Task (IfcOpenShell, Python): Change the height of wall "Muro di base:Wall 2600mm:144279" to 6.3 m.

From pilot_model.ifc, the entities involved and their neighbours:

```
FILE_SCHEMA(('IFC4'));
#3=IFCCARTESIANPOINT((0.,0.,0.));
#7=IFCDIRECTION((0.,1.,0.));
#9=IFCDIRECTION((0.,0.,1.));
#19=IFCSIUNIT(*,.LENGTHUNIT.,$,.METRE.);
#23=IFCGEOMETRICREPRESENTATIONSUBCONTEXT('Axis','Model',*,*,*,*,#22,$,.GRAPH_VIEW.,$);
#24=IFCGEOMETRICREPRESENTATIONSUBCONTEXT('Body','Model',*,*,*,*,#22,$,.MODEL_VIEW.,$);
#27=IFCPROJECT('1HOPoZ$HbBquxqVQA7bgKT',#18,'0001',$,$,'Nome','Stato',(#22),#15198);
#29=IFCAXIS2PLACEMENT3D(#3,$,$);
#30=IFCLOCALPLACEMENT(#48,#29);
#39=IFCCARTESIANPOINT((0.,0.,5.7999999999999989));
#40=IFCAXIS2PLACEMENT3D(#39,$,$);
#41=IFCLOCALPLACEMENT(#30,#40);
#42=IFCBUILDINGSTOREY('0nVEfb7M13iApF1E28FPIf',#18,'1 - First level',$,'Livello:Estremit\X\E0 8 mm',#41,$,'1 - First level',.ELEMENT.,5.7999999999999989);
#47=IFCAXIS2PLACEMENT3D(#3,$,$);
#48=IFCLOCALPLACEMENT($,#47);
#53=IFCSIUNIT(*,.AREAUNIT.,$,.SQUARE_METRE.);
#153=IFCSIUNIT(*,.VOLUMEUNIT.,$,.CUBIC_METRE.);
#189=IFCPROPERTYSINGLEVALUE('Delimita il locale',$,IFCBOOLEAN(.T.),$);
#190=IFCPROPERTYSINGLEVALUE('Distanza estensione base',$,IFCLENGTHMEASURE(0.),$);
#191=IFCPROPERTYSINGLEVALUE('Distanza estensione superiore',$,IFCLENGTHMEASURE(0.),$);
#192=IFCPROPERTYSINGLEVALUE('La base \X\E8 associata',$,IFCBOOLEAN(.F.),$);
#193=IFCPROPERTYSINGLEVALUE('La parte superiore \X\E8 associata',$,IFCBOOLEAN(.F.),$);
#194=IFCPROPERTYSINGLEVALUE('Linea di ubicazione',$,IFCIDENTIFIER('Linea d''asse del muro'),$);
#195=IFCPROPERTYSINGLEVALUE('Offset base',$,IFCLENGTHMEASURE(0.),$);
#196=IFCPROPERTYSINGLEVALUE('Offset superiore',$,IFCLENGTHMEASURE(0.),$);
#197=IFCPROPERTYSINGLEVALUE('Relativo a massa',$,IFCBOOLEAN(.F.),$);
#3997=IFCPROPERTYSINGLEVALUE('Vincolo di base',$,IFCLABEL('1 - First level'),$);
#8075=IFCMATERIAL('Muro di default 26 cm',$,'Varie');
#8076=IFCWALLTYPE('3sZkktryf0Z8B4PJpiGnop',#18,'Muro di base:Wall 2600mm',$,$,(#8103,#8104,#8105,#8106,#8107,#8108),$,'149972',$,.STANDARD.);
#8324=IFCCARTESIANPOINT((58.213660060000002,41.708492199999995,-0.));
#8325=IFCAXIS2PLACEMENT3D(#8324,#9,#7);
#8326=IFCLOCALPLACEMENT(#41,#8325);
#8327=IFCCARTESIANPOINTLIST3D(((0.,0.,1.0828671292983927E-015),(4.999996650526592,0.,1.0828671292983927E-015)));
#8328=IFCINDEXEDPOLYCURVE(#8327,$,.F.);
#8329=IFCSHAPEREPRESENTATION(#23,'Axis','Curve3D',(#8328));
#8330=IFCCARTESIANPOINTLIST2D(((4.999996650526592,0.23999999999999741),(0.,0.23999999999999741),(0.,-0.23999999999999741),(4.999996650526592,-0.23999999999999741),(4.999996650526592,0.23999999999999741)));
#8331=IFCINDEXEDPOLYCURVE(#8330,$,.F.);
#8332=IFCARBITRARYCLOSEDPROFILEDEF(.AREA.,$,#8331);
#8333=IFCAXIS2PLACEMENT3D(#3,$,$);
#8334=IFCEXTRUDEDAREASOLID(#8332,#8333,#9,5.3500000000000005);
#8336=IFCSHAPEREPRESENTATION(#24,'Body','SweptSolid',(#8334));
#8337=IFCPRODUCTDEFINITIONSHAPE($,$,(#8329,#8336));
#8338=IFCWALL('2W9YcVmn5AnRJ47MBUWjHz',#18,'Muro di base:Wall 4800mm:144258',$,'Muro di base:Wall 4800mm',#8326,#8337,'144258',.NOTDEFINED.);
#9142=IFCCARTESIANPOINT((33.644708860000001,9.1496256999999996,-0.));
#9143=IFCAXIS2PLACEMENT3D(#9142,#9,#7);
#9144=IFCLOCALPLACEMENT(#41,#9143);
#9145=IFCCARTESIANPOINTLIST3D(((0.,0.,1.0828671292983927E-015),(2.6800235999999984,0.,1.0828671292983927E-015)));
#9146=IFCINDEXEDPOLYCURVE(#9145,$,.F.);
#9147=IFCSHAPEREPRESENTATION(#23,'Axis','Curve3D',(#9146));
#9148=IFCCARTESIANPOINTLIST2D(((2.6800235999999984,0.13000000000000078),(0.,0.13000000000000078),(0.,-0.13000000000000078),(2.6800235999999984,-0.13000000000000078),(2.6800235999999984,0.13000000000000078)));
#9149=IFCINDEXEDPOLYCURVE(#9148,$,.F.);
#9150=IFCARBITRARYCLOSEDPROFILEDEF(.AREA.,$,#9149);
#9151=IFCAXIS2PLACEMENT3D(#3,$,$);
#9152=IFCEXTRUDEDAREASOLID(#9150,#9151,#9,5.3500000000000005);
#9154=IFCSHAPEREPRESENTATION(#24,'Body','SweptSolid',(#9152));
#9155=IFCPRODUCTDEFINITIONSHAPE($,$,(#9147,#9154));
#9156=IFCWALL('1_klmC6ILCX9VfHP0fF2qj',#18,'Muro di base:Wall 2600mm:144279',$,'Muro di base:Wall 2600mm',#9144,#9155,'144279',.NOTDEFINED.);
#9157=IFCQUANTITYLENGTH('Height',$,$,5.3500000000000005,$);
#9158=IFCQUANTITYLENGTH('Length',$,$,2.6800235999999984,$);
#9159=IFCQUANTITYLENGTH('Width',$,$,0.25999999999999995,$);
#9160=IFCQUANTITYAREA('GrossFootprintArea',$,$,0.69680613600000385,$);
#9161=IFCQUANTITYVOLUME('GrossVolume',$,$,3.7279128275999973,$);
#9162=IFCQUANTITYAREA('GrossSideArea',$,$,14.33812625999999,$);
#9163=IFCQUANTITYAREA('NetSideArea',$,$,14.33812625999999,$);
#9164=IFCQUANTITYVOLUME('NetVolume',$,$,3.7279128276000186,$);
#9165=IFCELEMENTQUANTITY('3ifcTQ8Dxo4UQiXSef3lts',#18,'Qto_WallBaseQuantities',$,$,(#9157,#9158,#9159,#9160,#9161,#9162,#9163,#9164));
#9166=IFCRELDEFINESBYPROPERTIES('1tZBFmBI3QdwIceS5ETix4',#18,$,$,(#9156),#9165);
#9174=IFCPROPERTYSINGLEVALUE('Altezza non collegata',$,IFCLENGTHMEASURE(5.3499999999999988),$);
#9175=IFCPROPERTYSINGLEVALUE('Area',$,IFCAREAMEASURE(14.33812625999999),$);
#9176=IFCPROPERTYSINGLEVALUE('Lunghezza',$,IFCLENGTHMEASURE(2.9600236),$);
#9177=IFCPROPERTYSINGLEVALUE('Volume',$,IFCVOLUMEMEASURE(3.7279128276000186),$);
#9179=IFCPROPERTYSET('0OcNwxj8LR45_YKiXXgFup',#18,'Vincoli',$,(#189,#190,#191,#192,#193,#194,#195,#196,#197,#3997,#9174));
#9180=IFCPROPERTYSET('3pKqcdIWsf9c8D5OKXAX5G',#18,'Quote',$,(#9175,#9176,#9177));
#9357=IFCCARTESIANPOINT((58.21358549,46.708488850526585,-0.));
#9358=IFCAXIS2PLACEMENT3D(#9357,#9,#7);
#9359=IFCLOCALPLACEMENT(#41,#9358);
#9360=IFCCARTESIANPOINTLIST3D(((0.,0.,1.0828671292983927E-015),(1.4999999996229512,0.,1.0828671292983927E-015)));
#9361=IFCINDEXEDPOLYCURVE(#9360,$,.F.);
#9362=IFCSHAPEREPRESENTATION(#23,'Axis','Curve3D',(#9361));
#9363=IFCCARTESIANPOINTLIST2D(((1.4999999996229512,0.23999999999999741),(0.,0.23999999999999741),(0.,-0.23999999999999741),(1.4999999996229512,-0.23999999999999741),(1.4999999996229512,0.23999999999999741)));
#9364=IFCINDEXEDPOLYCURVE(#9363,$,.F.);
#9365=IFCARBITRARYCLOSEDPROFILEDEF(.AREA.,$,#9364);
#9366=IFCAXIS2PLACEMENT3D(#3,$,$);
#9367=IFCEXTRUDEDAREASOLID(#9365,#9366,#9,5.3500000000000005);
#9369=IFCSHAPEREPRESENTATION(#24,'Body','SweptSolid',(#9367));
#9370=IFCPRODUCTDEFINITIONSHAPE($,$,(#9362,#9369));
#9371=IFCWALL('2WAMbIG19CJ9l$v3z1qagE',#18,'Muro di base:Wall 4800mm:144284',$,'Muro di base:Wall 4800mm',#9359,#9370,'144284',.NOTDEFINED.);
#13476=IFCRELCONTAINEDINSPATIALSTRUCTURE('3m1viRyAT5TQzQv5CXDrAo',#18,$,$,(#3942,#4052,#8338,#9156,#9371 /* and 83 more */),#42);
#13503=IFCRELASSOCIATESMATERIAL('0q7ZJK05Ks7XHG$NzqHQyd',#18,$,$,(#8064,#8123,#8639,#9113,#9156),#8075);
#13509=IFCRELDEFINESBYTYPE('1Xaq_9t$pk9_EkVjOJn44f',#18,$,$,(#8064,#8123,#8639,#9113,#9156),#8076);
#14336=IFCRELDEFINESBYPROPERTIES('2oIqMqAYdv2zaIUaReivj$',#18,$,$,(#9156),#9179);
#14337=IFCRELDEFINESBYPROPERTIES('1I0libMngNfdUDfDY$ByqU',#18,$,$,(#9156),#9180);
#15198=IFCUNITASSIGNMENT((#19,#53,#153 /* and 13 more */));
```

```python
import ifcopenshell
import ifcopenshell.api.pset
import ifcopenshell.geom
import ifcopenshell.util.element
import ifcopenshell.util.representation
import ifcopenshell.util.shape
import ifcopenshell.util.unit

model = ifcopenshell.open("pilot_model.ifc")
unit_scale = ifcopenshell.util.unit.calculate_unit_scale(model)
area_scale = ifcopenshell.util.unit.calculate_unit_scale(model, "AREAUNIT")
volume_scale = ifcopenshell.util.unit.calculate_unit_scale(model, "VOLUMEUNIT")
settings = ifcopenshell.geom.settings()


def volume(element):
    """Net volume in cubic metres, openings subtracted."""
    shape = ifcopenshell.geom.create_shape(settings, element)
    return ifcopenshell.util.shape.get_volume(shape.geometry)


wall = model.by_guid("1_klmC6ILCX9VfHP0fF2qj")
before = volume(wall)

body = ifcopenshell.util.representation.get_representation(wall, "Model", "Body")
solid = body.Items[0]
old_height = solid.Depth
solid.Depth = 6.3 / unit_scale
after = volume(wall)
thickness = 0.26  # wall thickness in metres

# Update the stored height, areas and volumes.
qto = model.by_id(ifcopenshell.util.element.get_pset(wall, "Qto_WallBaseQuantities", should_inherit=False)["id"])
ifcopenshell.api.pset.edit_qto(model, qto=qto, properties={
    "Height": solid.Depth,
    "GrossVolume": ifcopenshell.util.element.get_pset(wall, "Qto_WallBaseQuantities", "GrossVolume") * solid.Depth / old_height,
    "GrossSideArea": ifcopenshell.util.element.get_pset(wall, "Qto_WallBaseQuantities", "GrossSideArea") * solid.Depth / old_height,
    "NetSideArea": after / thickness / area_scale,
    "NetVolume": after / volume_scale,
})
pset = model.by_id(ifcopenshell.util.element.get_pset(wall, "Vincoli", should_inherit=False)["id"])
ifcopenshell.api.pset.edit_pset(model, pset=pset, properties={
    "Altezza non collegata": model.create_entity("IfcLengthMeasure", solid.Depth),
})
pset = model.by_id(ifcopenshell.util.element.get_pset(wall, "Quote", should_inherit=False)["id"])
ifcopenshell.api.pset.edit_pset(model, pset=pset, properties={
    "Area": model.create_entity("IfcAreaMeasure", after / thickness / area_scale),
    "Volume": model.create_entity("IfcVolumeMeasure", after / volume_scale),
})

print(f"height {old_height:g} -> {solid.Depth:g}, volume {before:.3f} -> {after:.3f} m3")

model.write("pilot_model-out.ifc")
```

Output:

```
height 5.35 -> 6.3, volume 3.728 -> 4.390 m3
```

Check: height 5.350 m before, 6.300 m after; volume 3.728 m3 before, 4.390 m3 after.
